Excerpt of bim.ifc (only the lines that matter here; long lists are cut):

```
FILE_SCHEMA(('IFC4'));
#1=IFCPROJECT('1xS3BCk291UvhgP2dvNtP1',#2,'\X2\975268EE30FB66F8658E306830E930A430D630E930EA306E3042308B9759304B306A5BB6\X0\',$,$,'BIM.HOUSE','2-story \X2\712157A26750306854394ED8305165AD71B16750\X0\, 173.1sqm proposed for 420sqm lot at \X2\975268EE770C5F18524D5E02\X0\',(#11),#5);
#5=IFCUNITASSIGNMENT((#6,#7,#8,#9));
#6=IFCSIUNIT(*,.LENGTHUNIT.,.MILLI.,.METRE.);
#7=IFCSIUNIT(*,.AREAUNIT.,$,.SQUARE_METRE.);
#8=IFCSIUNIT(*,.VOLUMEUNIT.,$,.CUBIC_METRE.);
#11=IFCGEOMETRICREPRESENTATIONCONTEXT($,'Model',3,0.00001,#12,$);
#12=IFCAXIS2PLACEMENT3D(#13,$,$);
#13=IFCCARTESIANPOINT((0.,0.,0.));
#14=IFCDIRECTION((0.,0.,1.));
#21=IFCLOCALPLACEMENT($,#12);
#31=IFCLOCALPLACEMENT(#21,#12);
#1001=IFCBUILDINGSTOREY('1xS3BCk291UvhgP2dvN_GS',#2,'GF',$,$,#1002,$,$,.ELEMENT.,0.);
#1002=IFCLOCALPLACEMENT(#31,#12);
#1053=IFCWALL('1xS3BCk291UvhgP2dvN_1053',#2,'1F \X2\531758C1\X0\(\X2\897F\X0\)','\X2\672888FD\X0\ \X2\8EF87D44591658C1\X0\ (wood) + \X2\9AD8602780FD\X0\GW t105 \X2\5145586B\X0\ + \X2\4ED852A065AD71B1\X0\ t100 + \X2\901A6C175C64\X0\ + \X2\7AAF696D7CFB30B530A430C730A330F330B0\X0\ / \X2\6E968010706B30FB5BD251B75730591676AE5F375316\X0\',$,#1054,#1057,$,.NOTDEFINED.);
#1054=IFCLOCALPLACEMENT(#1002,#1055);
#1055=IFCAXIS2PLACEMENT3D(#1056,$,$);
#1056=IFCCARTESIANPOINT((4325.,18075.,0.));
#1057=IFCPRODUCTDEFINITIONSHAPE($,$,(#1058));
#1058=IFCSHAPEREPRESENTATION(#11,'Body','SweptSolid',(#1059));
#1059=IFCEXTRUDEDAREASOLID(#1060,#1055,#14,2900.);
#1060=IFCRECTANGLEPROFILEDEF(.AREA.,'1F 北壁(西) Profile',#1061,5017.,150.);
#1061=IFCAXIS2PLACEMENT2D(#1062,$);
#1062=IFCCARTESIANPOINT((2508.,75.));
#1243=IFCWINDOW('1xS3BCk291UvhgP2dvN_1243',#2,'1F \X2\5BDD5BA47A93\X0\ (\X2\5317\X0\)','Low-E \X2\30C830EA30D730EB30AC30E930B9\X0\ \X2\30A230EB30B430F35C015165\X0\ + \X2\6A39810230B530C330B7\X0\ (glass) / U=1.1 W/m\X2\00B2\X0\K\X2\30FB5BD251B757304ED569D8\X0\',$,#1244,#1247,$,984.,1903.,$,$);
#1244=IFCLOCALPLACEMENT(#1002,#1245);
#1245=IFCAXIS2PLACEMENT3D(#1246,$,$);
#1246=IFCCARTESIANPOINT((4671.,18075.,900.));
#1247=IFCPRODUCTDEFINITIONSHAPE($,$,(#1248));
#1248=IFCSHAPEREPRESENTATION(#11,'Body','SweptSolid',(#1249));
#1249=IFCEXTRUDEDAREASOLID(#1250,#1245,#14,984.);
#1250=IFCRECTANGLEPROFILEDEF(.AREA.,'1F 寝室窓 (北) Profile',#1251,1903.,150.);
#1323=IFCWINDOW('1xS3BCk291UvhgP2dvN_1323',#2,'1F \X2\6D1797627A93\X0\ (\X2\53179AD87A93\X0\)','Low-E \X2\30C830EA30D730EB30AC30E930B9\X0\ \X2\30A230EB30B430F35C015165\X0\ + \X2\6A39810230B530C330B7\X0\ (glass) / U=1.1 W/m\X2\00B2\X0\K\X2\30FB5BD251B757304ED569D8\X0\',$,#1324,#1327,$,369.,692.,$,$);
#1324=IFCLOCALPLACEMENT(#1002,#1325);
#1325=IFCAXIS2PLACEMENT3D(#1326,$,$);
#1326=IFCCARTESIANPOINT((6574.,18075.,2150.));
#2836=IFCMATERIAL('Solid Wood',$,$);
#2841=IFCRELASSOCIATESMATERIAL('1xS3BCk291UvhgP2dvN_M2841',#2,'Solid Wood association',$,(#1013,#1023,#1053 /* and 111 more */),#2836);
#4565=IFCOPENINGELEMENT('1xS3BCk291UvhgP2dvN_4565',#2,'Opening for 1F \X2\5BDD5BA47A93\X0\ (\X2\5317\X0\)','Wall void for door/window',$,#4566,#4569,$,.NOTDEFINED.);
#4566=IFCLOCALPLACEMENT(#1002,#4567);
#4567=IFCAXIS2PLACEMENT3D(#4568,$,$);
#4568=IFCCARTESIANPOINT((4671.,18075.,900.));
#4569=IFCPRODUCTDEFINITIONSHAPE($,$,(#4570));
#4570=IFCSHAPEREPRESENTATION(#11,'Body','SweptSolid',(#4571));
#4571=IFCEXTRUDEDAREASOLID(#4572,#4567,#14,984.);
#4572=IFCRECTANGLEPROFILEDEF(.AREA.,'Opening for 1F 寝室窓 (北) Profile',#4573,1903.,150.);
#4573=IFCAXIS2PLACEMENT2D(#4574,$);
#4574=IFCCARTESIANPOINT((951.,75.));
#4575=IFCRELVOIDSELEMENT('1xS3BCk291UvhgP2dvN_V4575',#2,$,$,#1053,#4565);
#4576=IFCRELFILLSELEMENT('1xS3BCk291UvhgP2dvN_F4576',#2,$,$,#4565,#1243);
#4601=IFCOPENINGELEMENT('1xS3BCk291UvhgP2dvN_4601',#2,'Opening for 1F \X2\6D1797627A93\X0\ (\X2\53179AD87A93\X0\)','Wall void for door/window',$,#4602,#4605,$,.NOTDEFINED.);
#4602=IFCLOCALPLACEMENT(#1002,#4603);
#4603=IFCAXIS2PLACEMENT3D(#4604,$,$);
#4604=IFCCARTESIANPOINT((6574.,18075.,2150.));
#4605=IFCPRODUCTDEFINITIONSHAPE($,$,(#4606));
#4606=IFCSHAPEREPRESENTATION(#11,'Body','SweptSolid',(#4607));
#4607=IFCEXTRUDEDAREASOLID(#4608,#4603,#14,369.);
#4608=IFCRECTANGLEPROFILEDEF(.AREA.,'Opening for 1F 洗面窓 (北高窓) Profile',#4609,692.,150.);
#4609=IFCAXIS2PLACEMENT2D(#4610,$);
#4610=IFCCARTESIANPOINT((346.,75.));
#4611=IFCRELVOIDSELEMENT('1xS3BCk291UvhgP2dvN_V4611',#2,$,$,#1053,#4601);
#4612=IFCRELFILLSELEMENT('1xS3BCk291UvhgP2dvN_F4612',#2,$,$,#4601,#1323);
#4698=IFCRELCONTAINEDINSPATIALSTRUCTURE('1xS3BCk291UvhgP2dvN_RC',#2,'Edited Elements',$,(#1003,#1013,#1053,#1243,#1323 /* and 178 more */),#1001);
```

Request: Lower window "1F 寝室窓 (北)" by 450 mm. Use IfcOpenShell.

```python
import numpy as np
import ifcopenshell
import ifcopenshell.api.geometry
import ifcopenshell.util.placement
import ifcopenshell.util.unit

model = ifcopenshell.open("bim.ifc")
unit_scale = ifcopenshell.util.unit.calculate_unit_scale(model)

window = model.by_id(1243)
opening = window.FillsVoids[0].RelatingOpeningElement
dz = -0.45 / unit_scale

shift = np.array([0.0, 0.0, dz])
# The window is not placed relative to its opening, so move both.
for product in (opening, window):
    matrix = ifcopenshell.util.placement.get_local_placement(product.ObjectPlacement)
    matrix[:3, 3] += shift
    ifcopenshell.api.geometry.edit_object_placement(model, product=product, matrix=matrix, is_si=False)

print(f"moved by {dz * unit_scale:+.3f} m")

model.write("bim-out.ifc")
```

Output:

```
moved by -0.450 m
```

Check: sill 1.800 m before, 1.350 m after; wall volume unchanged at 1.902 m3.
